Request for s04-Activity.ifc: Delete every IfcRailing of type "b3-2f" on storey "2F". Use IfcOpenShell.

First a look at what the model holds.

```python
import ifcopenshell
import ifcopenshell.util.element

model = ifcopenshell.open("s04-Activity.ifc")
print(model.schema)
storey = next(s for s in model.by_type("IfcBuildingStorey") if s.Name == "2F")
railings = [e for e in ifcopenshell.util.element.get_decomposition(storey) if e.is_a("IfcRailing")]
seen = {}
for e in railings:
    element_type = ifcopenshell.util.element.get_type(e)
    name = element_type.Name if element_type not in (None, e) else None
    seen[name] = seen.get(name, 0) + 1
for name, count in sorted(seen.items(), key=str):
    print(count, "x", name)
```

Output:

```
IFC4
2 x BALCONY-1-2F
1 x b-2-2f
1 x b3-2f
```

```python
import ifcopenshell
import ifcopenshell.api.root
import ifcopenshell.util.element

model = ifcopenshell.open("s04-Activity.ifc")

storey = next(s for s in model.by_type("IfcBuildingStorey") if s.Name == "2F")
railings = [e for e in ifcopenshell.util.element.get_decomposition(storey) if e.is_a("IfcRailing")]
targets = [e for e in railings if (t := ifcopenshell.util.element.get_type(e)) not in (None, e) and t.Name == "b3-2f"]

for e in targets:
    ifcopenshell.api.root.remove_product(model, product=e)
print(len(targets), "removed")

model.write("s04-Activity_rev.ifc")
```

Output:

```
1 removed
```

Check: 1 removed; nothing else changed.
